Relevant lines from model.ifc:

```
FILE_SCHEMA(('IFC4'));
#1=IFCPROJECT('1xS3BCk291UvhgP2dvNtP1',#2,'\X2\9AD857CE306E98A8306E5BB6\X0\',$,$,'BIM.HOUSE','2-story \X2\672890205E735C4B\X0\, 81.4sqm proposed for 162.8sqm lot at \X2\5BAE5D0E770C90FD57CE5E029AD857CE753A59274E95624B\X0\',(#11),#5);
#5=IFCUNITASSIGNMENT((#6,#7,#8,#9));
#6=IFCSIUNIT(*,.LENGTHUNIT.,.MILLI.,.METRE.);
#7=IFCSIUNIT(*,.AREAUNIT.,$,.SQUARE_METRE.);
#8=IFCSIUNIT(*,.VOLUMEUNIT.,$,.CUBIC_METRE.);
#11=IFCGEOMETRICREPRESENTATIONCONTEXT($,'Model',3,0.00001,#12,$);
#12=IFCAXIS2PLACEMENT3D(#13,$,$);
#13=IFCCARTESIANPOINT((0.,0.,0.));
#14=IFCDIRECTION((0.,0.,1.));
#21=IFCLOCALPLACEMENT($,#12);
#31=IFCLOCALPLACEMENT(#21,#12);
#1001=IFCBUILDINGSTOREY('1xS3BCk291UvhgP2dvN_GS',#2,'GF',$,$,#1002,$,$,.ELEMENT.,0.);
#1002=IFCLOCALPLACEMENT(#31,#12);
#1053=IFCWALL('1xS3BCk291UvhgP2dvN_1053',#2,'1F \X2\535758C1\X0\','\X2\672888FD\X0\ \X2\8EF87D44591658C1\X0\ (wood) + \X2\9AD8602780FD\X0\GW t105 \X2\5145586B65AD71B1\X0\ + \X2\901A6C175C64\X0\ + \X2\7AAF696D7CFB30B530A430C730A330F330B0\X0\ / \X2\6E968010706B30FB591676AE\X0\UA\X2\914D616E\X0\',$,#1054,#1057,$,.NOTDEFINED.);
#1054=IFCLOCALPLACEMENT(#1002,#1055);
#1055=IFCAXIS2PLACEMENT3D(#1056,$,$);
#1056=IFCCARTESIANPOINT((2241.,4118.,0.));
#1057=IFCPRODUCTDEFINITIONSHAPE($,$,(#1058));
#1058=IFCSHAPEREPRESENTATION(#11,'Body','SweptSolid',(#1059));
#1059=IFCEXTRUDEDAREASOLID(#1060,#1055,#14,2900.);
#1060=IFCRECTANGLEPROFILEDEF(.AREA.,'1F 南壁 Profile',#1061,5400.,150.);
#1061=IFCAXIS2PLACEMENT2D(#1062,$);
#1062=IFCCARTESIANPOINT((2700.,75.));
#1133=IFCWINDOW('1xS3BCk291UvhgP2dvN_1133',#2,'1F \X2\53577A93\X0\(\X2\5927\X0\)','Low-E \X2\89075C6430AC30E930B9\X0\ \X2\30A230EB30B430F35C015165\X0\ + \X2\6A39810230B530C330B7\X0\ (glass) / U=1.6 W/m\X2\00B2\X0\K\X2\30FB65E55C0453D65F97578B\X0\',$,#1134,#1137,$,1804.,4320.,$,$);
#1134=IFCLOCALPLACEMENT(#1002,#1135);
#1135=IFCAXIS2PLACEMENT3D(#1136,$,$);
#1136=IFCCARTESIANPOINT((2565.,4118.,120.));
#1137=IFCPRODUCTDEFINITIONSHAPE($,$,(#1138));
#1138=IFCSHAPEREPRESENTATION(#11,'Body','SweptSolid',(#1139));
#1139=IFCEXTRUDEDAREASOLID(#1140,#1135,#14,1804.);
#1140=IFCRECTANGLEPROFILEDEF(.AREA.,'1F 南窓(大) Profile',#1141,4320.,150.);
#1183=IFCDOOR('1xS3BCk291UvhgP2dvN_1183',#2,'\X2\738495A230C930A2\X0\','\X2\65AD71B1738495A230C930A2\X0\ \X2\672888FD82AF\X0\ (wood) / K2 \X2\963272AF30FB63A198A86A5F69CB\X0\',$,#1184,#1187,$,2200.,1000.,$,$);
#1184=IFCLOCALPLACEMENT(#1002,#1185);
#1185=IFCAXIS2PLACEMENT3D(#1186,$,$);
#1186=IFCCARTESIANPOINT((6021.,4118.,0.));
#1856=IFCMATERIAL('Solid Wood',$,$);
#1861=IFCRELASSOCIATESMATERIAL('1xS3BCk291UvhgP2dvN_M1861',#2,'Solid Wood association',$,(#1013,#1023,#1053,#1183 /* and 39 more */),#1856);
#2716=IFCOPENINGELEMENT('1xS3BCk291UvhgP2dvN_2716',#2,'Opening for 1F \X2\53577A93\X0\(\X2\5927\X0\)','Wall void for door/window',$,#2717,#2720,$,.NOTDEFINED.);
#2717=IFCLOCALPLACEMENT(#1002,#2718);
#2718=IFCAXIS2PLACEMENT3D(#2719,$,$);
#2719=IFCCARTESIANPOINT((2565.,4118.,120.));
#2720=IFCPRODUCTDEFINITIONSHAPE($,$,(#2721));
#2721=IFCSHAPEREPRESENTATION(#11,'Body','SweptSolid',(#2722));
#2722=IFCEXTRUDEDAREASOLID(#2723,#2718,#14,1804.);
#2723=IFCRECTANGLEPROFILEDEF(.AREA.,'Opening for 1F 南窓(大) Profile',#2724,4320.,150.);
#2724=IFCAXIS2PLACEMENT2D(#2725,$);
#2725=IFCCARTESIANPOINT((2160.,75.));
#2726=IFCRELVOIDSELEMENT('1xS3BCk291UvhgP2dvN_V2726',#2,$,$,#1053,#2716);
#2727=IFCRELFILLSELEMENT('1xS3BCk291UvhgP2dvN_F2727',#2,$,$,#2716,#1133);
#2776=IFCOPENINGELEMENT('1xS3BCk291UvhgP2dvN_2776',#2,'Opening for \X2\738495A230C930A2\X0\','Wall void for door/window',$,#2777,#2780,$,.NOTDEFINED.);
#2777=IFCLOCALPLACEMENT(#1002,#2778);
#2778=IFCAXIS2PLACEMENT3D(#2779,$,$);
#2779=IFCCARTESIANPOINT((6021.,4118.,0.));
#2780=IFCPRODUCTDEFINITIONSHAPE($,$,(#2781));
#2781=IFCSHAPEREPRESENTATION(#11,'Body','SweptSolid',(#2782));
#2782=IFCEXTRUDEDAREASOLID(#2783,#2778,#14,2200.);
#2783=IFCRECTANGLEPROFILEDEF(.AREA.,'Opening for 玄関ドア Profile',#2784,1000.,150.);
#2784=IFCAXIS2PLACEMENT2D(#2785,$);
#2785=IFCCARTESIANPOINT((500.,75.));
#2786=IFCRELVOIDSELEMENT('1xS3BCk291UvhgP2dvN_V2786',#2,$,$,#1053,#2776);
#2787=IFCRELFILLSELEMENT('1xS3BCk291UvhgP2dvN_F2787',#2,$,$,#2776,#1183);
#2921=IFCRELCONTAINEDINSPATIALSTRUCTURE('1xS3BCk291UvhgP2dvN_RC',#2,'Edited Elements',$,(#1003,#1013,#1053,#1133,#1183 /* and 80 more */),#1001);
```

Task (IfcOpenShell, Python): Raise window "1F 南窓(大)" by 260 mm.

```python
import numpy as np
import ifcopenshell
import ifcopenshell.api.geometry
import ifcopenshell.util.placement
import ifcopenshell.util.unit

model = ifcopenshell.open("model.ifc")
unit_scale = ifcopenshell.util.unit.calculate_unit_scale(model)

window = model.by_id(1133)
opening = window.FillsVoids[0].RelatingOpeningElement
dz = 0.26 / unit_scale

shift = np.array([0.0, 0.0, dz])
# The window is not placed relative to its opening, so move both.
for product in (opening, window):
    matrix = ifcopenshell.util.placement.get_local_placement(product.ObjectPlacement)
    matrix[:3, 3] += shift
    ifcopenshell.api.geometry.edit_object_placement(model, product=product, matrix=matrix, is_si=False)

print(f"moved by {dz * unit_scale:+.3f} m")

model.write("model_v2.ifc")
```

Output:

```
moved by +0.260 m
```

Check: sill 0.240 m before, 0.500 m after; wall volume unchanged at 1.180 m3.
